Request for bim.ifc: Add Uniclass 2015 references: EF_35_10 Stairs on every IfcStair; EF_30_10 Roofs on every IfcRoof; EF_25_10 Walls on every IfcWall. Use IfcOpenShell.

First a look at what the model holds.

```python
import ifcopenshell

model = ifcopenshell.open("bim.ifc")
print(model.schema)
print("classifications:", [c.Name for c in model.by_type("IfcClassification")])
for ifc_class in ("IfcDoor", "IfcRoof", "IfcStair", "IfcWall", "IfcWindow"):
    print(ifc_class, len(model.by_type(ifc_class)))
```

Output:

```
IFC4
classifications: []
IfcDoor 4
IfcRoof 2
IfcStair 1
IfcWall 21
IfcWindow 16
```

```python
import ifcopenshell
import ifcopenshell.api.classification

model = ifcopenshell.open("bim.ifc")

system = ifcopenshell.api.classification.add_classification(model, classification="Uniclass 2015")

codes = {
    "IfcStair": ("EF_35_10", "Stairs"),
    "IfcRoof": ("EF_30_10", "Roofs"),
    "IfcWall": ("EF_25_10", "Walls"),
}
for ifc_class, (code, name) in codes.items():
    products = model.by_type(ifc_class)
    ifcopenshell.api.classification.add_reference(
        model, products=products, classification=system, identification=code, name=name
    )
    print(code, len(products))

model.write("bim_updated.ifc")
```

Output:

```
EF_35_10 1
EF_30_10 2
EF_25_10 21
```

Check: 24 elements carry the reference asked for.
